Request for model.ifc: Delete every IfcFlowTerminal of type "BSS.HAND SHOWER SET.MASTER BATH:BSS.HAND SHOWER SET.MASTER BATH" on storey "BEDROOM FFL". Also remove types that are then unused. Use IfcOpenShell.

First a look at what the model holds.

```python
import ifcopenshell
import ifcopenshell.util.element

model = ifcopenshell.open("model.ifc")
print(model.schema)
storey = next(s for s in model.by_type("IfcBuildingStorey") if s.Name == "BEDROOM FFL")
terminals = [e for e in ifcopenshell.util.element.get_decomposition(storey) if e.is_a("IfcFlowTerminal")]
seen = {}
for e in terminals:
    element_type = ifcopenshell.util.element.get_type(e)
    name = element_type.Name if element_type not in (None, e) else None
    seen[name] = seen.get(name, 0) + 1
for name, count in sorted(seen.items(), key=str):
    print(count, "x", name)
```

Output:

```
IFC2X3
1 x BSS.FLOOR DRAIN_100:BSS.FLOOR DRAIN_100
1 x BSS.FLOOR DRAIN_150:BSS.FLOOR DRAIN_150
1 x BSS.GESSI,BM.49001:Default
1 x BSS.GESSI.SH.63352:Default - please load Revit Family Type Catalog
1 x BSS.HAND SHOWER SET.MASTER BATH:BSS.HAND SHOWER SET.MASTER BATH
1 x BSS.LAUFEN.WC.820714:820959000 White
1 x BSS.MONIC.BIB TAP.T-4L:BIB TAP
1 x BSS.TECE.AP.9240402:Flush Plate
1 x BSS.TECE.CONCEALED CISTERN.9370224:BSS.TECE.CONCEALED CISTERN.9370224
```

```python
import ifcopenshell
import ifcopenshell.api.root
import ifcopenshell.util.element

model = ifcopenshell.open("model.ifc")

storey = next(s for s in model.by_type("IfcBuildingStorey") if s.Name == "BEDROOM FFL")
terminals = [e for e in ifcopenshell.util.element.get_decomposition(storey) if e.is_a("IfcFlowTerminal")]
targets = [e for e in terminals if (t := ifcopenshell.util.element.get_type(e)) not in (None, e) and t.Name == "BSS.HAND SHOWER SET.MASTER BATH:BSS.HAND SHOWER SET.MASTER BATH"]
types = {ifcopenshell.util.element.get_type(e) for e in targets} - {None, *targets}

for e in targets:
    ifcopenshell.api.root.remove_product(model, product=e)
print(len(targets), "removed")

unused = [t for t in types if not ifcopenshell.util.element.get_types(t)]
for t in unused:
    ifcopenshell.api.root.remove_product(model, product=t)
print(len(unused), "unused types removed")

model.write("model_updated.ifc")
```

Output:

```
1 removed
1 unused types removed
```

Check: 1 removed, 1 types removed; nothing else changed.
